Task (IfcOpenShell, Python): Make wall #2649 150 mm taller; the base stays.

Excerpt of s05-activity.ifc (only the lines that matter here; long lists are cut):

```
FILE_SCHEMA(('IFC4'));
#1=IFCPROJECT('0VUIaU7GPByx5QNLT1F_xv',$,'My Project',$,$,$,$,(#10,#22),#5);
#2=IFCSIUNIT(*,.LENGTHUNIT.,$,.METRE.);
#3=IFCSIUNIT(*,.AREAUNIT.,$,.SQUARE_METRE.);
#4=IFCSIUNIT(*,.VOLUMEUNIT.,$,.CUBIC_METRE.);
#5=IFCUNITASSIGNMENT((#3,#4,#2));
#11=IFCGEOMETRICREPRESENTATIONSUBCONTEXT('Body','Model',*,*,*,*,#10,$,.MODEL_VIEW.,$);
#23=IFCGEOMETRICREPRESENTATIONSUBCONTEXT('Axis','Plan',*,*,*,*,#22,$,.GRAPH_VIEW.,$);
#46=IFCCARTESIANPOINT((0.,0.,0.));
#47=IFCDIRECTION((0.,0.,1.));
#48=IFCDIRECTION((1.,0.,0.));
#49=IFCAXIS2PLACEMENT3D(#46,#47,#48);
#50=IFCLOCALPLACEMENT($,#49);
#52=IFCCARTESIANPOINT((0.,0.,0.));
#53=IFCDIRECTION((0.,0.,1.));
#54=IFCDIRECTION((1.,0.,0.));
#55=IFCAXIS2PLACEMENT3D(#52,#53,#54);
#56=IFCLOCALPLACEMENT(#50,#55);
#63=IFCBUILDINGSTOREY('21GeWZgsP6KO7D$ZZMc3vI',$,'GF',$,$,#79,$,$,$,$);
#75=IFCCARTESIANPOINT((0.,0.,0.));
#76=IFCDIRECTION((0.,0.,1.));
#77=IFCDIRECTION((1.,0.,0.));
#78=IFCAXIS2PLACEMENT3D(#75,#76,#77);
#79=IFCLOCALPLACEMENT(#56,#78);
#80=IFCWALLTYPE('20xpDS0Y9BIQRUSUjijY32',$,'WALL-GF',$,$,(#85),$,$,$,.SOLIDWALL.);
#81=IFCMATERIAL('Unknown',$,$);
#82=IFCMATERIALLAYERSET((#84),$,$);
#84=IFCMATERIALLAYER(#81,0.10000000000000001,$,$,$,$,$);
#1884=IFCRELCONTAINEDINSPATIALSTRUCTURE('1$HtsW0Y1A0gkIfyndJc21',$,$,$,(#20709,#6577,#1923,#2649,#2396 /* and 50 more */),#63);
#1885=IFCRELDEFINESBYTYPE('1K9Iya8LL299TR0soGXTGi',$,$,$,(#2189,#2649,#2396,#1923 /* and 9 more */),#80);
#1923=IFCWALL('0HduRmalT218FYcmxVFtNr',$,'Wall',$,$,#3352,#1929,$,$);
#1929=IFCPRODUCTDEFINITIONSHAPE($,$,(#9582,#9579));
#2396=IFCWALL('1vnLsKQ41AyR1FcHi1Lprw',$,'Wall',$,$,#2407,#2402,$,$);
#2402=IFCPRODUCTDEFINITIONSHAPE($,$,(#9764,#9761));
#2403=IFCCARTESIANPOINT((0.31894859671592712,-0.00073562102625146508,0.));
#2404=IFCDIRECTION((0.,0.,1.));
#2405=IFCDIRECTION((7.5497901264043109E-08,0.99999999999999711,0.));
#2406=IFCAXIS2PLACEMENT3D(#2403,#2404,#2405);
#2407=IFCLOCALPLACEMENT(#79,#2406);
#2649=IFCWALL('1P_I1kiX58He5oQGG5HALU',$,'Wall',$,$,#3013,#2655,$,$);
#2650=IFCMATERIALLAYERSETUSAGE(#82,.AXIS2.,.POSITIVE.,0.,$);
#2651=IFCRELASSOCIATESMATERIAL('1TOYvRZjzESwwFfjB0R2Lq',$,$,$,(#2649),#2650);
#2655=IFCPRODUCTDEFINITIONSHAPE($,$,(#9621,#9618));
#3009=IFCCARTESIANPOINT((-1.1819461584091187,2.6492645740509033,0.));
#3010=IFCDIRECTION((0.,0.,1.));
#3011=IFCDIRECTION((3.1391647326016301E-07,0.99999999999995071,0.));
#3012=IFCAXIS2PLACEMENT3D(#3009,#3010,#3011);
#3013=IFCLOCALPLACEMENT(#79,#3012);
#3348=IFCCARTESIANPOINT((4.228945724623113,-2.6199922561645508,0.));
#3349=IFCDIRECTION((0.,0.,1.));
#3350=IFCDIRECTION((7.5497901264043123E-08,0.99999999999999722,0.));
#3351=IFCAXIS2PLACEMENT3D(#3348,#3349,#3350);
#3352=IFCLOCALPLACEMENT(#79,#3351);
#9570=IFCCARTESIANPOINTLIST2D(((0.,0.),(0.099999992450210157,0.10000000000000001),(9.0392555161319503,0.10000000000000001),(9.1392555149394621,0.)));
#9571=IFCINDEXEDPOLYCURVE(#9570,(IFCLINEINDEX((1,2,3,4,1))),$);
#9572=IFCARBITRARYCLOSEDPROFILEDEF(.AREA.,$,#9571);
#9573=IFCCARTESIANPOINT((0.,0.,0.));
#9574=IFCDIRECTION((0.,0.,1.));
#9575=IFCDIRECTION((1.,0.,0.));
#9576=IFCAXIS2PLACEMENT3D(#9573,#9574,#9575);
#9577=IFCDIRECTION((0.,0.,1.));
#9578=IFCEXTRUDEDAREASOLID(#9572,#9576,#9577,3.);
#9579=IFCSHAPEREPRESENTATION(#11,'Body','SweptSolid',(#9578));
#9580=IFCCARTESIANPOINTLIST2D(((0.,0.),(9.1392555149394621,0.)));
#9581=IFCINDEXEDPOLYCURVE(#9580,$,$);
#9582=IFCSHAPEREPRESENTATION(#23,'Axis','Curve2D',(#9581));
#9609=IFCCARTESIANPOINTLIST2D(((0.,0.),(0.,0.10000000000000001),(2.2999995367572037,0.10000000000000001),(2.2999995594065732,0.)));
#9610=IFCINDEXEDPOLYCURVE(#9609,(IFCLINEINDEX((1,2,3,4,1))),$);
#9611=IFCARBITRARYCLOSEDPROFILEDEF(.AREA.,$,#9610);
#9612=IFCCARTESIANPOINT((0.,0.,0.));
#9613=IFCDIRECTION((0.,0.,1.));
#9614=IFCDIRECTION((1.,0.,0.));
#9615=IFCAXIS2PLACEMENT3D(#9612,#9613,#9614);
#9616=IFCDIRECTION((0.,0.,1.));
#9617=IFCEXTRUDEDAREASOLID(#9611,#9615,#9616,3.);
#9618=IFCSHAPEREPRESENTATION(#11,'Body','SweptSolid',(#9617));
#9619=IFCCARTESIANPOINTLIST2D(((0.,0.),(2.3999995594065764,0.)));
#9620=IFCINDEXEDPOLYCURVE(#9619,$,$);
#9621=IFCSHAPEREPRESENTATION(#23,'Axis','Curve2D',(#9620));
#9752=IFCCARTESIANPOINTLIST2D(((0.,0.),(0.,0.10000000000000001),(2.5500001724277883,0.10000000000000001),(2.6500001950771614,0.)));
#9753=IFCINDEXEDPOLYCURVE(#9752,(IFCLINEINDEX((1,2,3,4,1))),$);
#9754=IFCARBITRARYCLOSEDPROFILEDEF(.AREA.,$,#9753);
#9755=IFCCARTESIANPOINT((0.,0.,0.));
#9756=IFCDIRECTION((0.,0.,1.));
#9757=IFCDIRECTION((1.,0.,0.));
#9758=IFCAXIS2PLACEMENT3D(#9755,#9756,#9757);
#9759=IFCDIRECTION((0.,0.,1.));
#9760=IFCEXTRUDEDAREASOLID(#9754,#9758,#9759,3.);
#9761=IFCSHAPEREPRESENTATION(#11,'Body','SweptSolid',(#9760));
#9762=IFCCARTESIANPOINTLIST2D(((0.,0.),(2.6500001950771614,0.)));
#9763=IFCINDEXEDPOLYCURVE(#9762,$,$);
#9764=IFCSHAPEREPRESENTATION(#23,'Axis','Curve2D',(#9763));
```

```python
import ifcopenshell
import ifcopenshell.geom
import ifcopenshell.util.representation
import ifcopenshell.util.shape
import ifcopenshell.util.unit

model = ifcopenshell.open("s05-activity.ifc")
unit_scale = ifcopenshell.util.unit.calculate_unit_scale(model)
settings = ifcopenshell.geom.settings()


def volume(element):
    """Net volume in cubic metres, openings subtracted."""
    shape = ifcopenshell.geom.create_shape(settings, element)
    return ifcopenshell.util.shape.get_volume(shape.geometry)


wall = model.by_id(2649)
before = volume(wall)

body = ifcopenshell.util.representation.get_representation(wall, "Model", "Body")
solid = body.Items[0]
old_height = solid.Depth
solid.Depth += 0.15 / unit_scale
after = volume(wall)

print(f"height {old_height:g} -> {solid.Depth:g}, volume {before:.3f} -> {after:.3f} m3")

model.write("s05-activity_updated.ifc")
```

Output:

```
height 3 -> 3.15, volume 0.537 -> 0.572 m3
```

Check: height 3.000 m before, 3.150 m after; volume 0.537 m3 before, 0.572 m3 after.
